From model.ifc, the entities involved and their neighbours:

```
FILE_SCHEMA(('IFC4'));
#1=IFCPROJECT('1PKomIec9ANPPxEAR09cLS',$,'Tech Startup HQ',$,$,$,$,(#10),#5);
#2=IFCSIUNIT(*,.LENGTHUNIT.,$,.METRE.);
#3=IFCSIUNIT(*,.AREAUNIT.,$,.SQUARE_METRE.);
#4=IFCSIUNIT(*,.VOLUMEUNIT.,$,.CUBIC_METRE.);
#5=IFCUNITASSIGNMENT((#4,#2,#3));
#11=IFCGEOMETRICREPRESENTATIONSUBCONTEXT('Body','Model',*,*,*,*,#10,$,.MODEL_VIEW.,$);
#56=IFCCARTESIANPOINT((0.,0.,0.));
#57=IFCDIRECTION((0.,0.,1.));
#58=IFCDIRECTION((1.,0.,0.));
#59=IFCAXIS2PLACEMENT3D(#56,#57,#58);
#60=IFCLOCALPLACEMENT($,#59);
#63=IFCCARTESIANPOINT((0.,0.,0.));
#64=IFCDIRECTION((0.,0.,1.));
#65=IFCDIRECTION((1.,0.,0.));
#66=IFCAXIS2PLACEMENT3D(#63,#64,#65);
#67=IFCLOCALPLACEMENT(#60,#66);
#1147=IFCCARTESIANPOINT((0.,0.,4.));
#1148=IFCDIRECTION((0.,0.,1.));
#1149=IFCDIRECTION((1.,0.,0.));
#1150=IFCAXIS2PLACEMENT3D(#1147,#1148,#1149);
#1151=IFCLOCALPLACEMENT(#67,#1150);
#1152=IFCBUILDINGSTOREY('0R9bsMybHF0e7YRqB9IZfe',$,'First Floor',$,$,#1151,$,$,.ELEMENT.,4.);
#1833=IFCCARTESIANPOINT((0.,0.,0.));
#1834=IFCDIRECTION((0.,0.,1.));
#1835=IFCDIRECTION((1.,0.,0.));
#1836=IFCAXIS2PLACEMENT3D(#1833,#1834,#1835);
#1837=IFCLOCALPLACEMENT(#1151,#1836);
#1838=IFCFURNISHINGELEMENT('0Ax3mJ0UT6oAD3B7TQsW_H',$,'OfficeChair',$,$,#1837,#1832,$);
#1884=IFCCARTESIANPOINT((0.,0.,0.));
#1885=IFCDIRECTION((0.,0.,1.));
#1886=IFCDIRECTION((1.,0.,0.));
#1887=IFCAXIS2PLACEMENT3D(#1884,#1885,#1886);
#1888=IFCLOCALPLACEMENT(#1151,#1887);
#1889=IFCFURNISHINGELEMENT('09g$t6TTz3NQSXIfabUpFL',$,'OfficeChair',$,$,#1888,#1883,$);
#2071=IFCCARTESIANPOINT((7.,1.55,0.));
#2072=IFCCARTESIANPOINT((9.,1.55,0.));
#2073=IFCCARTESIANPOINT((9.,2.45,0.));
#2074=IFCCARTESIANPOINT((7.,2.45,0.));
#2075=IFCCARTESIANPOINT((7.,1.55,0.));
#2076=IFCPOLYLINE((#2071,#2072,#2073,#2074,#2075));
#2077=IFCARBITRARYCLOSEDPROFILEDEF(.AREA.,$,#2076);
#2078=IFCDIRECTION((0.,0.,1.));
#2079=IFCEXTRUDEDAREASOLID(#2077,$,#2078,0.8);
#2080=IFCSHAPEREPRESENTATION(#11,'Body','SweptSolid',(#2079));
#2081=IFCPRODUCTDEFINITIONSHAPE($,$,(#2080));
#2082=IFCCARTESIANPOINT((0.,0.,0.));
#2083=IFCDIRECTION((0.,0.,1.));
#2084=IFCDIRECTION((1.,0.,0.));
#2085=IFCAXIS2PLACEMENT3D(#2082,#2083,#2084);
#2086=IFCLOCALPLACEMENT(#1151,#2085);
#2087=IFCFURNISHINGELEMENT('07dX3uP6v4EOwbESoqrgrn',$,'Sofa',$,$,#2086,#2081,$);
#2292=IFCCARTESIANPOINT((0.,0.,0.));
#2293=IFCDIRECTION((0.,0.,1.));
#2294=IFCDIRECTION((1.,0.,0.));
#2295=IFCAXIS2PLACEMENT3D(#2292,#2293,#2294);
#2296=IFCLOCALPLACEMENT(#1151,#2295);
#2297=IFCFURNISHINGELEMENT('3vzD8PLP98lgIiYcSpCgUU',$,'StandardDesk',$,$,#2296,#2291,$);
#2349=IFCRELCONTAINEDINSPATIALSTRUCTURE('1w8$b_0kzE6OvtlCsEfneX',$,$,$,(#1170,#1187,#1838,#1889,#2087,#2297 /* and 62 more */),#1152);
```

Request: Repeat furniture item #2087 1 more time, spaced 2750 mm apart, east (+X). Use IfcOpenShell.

```python
import numpy as np
import ifcopenshell
import ifcopenshell.api.geometry
import ifcopenshell.api.root
import ifcopenshell.util.element
import ifcopenshell.util.placement

model = ifcopenshell.open("model.ifc")

source = model.by_id(2087)
base = ifcopenshell.util.placement.get_local_placement(source.ObjectPlacement)
step = np.array([1.0, 0.0, 0.0]) * 2.75

for i in range(1, 2):
    copy = ifcopenshell.api.root.copy_class(model, product=source)
    copy.Representation = ifcopenshell.util.element.copy_deep(
        model, source.Representation, exclude=["IfcGeometricRepresentationContext", "IfcRepresentationMap"]
    )
    matrix = base.copy()
    matrix[:3, 3] += i * step
    print("added at", matrix[:3, 3].round(3) + 0.0)
    ifcopenshell.api.geometry.edit_object_placement(model, product=copy, matrix=matrix, is_si=False)

model.write("model-out.ifc")
```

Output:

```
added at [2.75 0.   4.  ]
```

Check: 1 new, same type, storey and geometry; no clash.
